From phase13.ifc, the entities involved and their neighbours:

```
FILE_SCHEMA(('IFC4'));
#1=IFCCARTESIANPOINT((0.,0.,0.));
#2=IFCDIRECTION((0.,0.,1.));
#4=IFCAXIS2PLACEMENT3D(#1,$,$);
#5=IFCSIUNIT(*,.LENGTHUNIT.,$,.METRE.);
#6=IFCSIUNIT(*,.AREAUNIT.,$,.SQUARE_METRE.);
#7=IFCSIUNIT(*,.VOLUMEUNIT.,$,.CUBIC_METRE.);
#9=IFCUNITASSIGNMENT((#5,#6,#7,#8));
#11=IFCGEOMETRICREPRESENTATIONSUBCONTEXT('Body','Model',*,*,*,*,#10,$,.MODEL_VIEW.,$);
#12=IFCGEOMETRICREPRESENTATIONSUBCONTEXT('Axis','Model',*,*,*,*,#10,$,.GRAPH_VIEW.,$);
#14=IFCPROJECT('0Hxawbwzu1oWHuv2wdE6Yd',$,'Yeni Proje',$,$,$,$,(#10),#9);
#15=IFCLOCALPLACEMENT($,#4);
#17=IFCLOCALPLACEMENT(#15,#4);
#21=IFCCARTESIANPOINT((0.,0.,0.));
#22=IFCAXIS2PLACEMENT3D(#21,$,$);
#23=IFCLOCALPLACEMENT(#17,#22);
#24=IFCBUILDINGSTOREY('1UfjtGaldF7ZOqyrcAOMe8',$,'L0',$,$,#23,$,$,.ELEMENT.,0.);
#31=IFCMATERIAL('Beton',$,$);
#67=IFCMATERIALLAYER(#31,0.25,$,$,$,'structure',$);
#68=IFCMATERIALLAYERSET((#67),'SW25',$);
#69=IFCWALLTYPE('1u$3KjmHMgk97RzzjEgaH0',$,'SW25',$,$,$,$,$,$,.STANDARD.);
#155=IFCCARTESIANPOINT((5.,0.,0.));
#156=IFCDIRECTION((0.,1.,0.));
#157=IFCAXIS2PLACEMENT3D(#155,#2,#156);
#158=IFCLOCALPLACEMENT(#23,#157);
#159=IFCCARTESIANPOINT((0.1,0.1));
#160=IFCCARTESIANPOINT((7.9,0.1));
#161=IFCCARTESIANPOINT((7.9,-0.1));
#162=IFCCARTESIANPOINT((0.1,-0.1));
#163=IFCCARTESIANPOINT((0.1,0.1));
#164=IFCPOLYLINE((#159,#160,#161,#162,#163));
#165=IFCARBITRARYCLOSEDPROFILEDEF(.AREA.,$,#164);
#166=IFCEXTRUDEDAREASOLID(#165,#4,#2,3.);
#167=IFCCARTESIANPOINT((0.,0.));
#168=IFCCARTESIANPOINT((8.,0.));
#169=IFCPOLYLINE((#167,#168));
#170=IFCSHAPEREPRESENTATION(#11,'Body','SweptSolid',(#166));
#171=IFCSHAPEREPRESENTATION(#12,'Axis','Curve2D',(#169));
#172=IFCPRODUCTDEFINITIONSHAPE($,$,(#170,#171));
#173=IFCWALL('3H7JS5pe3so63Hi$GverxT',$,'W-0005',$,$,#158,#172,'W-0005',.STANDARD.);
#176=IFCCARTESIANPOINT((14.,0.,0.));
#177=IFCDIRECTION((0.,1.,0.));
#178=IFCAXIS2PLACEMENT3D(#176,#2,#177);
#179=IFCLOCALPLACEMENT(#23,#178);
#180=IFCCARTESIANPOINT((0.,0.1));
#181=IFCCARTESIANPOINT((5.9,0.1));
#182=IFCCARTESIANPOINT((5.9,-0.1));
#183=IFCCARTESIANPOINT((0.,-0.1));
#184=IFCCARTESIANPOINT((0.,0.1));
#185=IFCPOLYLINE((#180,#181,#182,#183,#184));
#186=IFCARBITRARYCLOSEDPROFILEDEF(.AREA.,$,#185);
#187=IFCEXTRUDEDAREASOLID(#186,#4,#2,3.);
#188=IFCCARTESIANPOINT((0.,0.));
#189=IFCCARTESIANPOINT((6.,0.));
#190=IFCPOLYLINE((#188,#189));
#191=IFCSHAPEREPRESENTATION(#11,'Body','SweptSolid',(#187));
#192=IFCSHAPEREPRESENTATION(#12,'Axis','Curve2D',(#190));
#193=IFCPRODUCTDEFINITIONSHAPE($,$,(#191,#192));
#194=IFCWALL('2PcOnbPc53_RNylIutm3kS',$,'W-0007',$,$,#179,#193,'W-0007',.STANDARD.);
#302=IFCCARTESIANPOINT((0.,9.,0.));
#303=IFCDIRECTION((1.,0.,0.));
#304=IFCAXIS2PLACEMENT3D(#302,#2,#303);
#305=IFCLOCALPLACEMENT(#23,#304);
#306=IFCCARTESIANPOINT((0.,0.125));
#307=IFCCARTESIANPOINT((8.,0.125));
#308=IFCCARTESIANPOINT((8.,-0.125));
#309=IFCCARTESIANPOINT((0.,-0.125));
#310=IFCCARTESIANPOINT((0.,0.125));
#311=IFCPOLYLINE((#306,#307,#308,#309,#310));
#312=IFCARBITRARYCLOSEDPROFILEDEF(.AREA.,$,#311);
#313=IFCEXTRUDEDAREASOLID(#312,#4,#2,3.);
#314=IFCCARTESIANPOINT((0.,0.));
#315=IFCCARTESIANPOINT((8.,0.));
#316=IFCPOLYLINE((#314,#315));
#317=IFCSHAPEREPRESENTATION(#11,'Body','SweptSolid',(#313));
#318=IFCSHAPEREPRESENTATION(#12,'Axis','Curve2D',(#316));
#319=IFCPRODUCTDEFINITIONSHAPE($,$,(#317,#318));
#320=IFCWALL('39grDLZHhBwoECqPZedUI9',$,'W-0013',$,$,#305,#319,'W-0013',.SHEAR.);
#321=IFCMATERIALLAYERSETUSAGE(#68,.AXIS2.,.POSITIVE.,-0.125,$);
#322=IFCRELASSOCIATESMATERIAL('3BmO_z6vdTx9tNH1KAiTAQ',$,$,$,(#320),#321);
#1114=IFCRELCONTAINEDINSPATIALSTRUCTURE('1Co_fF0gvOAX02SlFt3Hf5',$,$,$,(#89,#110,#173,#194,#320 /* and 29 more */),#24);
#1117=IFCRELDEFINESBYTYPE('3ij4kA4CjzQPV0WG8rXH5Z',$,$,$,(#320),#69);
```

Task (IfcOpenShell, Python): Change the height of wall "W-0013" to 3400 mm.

```python
import ifcopenshell
import ifcopenshell.geom
import ifcopenshell.util.representation
import ifcopenshell.util.shape
import ifcopenshell.util.unit

model = ifcopenshell.open("phase13.ifc")
unit_scale = ifcopenshell.util.unit.calculate_unit_scale(model)
settings = ifcopenshell.geom.settings()


def volume(element):
    """Net volume in cubic metres, openings subtracted."""
    shape = ifcopenshell.geom.create_shape(settings, element)
    return ifcopenshell.util.shape.get_volume(shape.geometry)


wall = model.by_guid("39grDLZHhBwoECqPZedUI9")
before = volume(wall)

body = ifcopenshell.util.representation.get_representation(wall, "Model", "Body")
solid = body.Items[0]
old_height = solid.Depth
solid.Depth = 3.4 / unit_scale
after = volume(wall)

print(f"height {old_height:g} -> {solid.Depth:g}, volume {before:.3f} -> {after:.3f} m3")

model.write("phase13_v2.ifc")
```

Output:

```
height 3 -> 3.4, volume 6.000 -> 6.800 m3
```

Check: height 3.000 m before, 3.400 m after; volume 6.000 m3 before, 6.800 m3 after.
